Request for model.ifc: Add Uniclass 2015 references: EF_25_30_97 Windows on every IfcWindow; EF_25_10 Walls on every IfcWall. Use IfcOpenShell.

First a look at what the model holds.

```python
import ifcopenshell

model = ifcopenshell.open("model.ifc")
print(model.schema)
print("classifications:", [c.Name for c in model.by_type("IfcClassification")])
for ifc_class in ("IfcDoor", "IfcRoof", "IfcStair", "IfcWall", "IfcWindow"):
    print(ifc_class, len(model.by_type(ifc_class)))
```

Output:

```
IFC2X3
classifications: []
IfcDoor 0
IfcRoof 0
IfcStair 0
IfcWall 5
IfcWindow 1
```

```python
import ifcopenshell
import ifcopenshell.api.classification

model = ifcopenshell.open("model.ifc")

# IFC2X3 requires Source and Edition and has no link from the project to the system.
system = model.create_entity("IfcClassification", Source="NBS", Edition="2015", Name="Uniclass 2015")

codes = {
    "IfcWindow": ("EF_25_30_97", "Windows"),
    "IfcWall": ("EF_25_10", "Walls"),
}
for ifc_class, (code, name) in codes.items():
    products = model.by_type(ifc_class)
    ifcopenshell.api.classification.add_reference(
        model, products=products, classification=system, identification=code, name=name
    )
    print(code, len(products))

model.write("model_v2.ifc")
```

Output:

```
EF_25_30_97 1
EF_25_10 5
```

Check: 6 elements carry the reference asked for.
